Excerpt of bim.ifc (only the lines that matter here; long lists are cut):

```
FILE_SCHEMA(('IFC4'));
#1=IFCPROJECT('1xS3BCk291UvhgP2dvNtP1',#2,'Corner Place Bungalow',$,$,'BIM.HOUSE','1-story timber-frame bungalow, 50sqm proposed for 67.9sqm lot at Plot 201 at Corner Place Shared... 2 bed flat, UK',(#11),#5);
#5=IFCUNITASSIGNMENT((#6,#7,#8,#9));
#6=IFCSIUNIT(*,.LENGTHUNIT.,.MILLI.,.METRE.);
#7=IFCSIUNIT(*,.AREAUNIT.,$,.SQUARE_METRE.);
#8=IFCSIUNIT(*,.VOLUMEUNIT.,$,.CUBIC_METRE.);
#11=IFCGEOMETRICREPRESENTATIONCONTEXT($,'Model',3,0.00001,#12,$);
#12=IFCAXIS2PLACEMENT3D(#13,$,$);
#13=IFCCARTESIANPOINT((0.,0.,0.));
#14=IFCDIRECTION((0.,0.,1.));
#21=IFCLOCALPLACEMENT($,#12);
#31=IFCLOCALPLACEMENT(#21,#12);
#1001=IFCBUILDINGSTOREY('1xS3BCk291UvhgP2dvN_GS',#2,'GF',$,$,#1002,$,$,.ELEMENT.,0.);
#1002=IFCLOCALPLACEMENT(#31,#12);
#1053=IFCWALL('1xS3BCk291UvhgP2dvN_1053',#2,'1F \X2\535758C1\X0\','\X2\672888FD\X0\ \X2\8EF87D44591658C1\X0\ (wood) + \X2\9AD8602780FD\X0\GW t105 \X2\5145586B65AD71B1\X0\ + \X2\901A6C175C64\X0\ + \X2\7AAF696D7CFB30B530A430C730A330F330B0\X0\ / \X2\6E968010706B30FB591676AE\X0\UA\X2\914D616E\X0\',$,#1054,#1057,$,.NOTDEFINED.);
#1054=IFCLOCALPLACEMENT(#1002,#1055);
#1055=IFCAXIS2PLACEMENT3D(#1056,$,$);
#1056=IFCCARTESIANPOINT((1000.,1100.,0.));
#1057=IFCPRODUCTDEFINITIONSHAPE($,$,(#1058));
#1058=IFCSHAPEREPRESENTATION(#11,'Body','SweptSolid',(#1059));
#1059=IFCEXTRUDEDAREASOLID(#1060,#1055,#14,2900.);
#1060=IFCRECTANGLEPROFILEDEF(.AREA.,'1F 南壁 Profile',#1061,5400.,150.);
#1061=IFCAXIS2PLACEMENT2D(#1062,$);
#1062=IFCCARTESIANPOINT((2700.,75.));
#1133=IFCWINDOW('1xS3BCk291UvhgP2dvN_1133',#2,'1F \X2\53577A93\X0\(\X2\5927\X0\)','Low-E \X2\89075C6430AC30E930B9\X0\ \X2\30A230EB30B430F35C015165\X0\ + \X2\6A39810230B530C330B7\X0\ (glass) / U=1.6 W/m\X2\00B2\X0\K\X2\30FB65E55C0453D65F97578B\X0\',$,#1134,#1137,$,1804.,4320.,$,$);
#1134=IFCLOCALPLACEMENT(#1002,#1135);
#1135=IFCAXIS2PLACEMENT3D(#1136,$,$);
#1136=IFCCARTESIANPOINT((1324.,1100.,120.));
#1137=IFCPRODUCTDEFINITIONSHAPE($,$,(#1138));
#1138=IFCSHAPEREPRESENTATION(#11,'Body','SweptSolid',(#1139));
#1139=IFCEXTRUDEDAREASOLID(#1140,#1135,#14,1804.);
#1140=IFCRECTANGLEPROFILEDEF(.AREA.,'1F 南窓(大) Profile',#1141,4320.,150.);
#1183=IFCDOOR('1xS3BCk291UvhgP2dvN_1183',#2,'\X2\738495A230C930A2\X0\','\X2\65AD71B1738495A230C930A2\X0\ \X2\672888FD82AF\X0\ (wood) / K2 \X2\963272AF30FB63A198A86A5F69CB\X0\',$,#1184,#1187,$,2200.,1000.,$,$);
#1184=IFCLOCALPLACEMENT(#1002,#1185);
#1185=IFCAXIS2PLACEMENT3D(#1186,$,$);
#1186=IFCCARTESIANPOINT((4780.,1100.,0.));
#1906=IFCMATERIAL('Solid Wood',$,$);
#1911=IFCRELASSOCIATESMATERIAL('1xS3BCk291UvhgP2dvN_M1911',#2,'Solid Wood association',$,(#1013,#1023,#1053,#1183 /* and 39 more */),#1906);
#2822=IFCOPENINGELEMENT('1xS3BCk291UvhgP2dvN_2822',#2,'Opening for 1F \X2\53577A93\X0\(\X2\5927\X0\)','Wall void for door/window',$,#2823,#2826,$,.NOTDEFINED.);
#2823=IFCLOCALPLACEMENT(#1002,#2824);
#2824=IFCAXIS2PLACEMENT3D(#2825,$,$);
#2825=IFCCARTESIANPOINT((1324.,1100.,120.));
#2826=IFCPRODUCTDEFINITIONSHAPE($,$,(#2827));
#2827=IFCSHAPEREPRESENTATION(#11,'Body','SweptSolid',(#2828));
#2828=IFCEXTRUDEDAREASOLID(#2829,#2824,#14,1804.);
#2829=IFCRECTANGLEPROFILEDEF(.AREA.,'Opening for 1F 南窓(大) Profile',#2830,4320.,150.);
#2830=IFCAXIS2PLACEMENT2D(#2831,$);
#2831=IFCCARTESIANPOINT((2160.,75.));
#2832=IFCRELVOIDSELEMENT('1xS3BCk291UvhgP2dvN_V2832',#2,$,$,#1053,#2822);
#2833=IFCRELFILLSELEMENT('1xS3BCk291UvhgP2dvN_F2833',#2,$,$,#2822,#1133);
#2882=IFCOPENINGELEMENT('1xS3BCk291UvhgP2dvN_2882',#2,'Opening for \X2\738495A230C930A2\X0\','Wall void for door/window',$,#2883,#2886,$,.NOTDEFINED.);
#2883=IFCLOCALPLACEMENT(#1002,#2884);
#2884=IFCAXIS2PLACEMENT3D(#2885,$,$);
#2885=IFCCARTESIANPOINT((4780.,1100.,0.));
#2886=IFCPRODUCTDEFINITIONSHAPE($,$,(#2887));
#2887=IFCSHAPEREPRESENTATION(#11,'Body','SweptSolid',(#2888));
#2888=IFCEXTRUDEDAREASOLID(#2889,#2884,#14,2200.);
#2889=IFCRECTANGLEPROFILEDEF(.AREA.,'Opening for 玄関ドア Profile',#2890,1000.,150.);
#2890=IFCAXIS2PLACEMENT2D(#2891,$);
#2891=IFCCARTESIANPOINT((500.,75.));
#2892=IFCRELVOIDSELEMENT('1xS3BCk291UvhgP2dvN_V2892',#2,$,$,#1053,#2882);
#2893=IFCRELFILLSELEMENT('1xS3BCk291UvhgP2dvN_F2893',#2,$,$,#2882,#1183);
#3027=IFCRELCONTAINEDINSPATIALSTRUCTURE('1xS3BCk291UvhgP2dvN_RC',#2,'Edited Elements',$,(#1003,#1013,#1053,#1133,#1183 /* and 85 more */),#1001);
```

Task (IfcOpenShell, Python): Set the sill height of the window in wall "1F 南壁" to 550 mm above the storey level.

```python
import numpy as np
import ifcopenshell
import ifcopenshell.api.geometry
import ifcopenshell.geom
import ifcopenshell.util.element
import ifcopenshell.util.placement
import ifcopenshell.util.shape
import ifcopenshell.util.unit

model = ifcopenshell.open("bim.ifc")
unit_scale = ifcopenshell.util.unit.calculate_unit_scale(model)

window = model.by_guid("1xS3BCk291UvhgP2dvN_1133")
opening = window.FillsVoids[0].RelatingOpeningElement
storey = ifcopenshell.util.element.get_container(window, ifc_class="IfcBuildingStorey")
level = ifcopenshell.util.placement.get_local_placement(storey.ObjectPlacement)[2, 3]

# The opening's origin need not be at the sill, so measure its lowest point.
shape = ifcopenshell.geom.create_shape(ifcopenshell.geom.settings(), opening)
bottom = ifcopenshell.util.shape.get_shape_bottom_elevation(shape, shape.geometry) / unit_scale
dz = level + 0.55 / unit_scale - bottom

shift = np.array([0.0, 0.0, dz])
# The window is not placed relative to its opening, so move both.
for product in (opening, window):
    matrix = ifcopenshell.util.placement.get_local_placement(product.ObjectPlacement)
    matrix[:3, 3] += shift
    ifcopenshell.api.geometry.edit_object_placement(model, product=product, matrix=matrix, is_si=False)

print(f"moved by {dz * unit_scale:+.3f} m")

model.write("bim_edited.ifc")
```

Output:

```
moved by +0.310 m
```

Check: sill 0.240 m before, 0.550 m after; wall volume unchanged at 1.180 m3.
